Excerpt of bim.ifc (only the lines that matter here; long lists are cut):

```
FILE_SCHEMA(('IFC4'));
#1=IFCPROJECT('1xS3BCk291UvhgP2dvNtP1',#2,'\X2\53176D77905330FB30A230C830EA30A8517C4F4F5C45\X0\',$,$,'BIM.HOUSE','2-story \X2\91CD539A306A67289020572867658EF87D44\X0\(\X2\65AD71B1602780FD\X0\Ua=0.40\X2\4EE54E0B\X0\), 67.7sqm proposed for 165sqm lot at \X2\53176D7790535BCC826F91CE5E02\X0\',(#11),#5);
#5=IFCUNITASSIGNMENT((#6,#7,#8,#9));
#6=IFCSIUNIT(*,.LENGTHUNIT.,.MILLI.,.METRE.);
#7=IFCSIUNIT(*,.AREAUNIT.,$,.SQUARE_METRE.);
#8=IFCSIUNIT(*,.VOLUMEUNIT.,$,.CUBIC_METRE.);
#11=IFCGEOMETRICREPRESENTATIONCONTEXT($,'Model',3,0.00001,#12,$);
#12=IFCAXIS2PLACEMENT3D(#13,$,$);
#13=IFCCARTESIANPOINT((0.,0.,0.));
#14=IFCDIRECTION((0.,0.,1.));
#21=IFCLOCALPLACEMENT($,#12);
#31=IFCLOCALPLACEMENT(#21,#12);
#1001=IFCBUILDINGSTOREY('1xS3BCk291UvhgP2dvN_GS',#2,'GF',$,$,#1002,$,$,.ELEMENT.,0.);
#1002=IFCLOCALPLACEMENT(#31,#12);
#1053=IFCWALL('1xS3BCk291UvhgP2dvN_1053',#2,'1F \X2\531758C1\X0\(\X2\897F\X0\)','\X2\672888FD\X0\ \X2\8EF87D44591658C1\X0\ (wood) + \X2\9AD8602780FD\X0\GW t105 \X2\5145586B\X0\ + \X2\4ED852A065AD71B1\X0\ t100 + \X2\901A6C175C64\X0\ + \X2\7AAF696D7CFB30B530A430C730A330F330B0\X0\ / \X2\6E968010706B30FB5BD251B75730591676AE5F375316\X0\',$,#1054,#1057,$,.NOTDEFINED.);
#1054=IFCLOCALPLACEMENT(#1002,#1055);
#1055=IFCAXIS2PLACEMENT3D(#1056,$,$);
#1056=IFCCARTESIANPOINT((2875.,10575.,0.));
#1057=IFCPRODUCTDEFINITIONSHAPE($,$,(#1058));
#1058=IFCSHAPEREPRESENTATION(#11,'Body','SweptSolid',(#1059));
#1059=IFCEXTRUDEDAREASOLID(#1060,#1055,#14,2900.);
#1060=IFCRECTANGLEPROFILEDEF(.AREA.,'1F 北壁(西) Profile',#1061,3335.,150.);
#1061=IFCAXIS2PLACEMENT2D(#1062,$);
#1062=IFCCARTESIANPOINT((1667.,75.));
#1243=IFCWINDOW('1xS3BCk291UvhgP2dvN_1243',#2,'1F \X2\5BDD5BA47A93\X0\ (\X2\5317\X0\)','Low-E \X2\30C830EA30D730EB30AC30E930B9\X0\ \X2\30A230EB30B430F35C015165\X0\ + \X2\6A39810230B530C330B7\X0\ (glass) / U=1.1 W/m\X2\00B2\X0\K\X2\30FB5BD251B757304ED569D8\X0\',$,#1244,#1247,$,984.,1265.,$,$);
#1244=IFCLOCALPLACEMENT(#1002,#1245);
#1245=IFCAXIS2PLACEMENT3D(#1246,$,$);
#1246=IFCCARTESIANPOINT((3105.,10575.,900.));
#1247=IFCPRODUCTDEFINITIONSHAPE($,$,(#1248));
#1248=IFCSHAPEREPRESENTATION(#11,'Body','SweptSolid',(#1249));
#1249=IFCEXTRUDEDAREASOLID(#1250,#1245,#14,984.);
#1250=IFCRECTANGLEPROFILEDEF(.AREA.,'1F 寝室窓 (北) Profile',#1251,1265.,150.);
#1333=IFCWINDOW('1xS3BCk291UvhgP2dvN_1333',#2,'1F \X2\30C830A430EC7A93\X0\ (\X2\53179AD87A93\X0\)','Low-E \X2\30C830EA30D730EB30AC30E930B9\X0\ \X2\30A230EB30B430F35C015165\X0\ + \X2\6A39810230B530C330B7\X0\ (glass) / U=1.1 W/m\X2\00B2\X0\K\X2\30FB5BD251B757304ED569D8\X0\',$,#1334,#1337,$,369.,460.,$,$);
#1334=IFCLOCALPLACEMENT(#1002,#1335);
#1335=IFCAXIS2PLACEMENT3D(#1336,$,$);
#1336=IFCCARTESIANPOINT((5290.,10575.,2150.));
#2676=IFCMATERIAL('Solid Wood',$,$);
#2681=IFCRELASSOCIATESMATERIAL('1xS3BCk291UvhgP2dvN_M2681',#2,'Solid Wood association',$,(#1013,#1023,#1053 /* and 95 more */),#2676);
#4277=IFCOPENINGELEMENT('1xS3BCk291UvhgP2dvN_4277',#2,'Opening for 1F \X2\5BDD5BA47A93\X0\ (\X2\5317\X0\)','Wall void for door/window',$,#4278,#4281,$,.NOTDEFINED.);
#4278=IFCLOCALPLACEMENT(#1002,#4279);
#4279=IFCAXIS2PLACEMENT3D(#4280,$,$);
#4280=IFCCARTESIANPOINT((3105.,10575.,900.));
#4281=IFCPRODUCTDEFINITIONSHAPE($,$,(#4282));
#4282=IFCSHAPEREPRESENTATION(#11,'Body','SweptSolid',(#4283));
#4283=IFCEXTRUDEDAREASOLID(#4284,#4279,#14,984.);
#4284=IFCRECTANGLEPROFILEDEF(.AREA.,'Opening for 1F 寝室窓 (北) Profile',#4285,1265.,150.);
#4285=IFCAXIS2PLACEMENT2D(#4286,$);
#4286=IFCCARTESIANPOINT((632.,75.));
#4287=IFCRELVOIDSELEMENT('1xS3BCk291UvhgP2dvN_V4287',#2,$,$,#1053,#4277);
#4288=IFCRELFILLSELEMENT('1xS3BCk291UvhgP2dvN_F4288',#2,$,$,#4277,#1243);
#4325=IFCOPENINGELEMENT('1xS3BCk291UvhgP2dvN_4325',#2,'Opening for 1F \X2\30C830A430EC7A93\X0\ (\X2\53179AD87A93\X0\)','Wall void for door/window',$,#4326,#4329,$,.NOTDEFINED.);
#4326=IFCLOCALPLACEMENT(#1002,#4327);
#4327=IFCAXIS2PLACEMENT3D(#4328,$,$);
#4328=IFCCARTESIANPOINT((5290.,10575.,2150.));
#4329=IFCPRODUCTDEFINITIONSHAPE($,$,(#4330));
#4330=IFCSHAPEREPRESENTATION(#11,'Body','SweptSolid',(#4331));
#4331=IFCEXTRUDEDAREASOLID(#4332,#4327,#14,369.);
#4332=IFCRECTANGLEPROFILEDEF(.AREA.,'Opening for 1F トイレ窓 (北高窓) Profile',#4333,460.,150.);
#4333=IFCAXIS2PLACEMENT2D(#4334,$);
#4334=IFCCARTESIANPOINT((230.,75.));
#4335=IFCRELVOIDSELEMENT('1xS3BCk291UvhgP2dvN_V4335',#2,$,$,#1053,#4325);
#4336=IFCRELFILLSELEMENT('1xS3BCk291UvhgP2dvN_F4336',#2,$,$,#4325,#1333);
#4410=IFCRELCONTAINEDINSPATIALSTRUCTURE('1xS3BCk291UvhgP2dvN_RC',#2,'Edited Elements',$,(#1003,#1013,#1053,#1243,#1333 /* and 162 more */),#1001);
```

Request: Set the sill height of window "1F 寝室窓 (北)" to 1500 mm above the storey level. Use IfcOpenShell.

```python
import numpy as np
import ifcopenshell
import ifcopenshell.api.geometry
import ifcopenshell.geom
import ifcopenshell.util.element
import ifcopenshell.util.placement
import ifcopenshell.util.shape
import ifcopenshell.util.unit

model = ifcopenshell.open("bim.ifc")
unit_scale = ifcopenshell.util.unit.calculate_unit_scale(model)

window = model.by_id(1243)
opening = window.FillsVoids[0].RelatingOpeningElement
storey = ifcopenshell.util.element.get_container(window, ifc_class="IfcBuildingStorey")
level = ifcopenshell.util.placement.get_local_placement(storey.ObjectPlacement)[2, 3]

# The opening's origin need not be at the sill, so measure its lowest point.
shape = ifcopenshell.geom.create_shape(ifcopenshell.geom.settings(), opening)
bottom = ifcopenshell.util.shape.get_shape_bottom_elevation(shape, shape.geometry) / unit_scale
dz = level + 1.5 / unit_scale - bottom

shift = np.array([0.0, 0.0, dz])
# The window is not placed relative to its opening, so move both.
for product in (opening, window):
    matrix = ifcopenshell.util.placement.get_local_placement(product.ObjectPlacement)
    matrix[:3, 3] += shift
    ifcopenshell.api.geometry.edit_object_placement(model, product=product, matrix=matrix, is_si=False)

print(f"moved by {dz * unit_scale:+.3f} m")

model.write("bim_updated.ifc")
```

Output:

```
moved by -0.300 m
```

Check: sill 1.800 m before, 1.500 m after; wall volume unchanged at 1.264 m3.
